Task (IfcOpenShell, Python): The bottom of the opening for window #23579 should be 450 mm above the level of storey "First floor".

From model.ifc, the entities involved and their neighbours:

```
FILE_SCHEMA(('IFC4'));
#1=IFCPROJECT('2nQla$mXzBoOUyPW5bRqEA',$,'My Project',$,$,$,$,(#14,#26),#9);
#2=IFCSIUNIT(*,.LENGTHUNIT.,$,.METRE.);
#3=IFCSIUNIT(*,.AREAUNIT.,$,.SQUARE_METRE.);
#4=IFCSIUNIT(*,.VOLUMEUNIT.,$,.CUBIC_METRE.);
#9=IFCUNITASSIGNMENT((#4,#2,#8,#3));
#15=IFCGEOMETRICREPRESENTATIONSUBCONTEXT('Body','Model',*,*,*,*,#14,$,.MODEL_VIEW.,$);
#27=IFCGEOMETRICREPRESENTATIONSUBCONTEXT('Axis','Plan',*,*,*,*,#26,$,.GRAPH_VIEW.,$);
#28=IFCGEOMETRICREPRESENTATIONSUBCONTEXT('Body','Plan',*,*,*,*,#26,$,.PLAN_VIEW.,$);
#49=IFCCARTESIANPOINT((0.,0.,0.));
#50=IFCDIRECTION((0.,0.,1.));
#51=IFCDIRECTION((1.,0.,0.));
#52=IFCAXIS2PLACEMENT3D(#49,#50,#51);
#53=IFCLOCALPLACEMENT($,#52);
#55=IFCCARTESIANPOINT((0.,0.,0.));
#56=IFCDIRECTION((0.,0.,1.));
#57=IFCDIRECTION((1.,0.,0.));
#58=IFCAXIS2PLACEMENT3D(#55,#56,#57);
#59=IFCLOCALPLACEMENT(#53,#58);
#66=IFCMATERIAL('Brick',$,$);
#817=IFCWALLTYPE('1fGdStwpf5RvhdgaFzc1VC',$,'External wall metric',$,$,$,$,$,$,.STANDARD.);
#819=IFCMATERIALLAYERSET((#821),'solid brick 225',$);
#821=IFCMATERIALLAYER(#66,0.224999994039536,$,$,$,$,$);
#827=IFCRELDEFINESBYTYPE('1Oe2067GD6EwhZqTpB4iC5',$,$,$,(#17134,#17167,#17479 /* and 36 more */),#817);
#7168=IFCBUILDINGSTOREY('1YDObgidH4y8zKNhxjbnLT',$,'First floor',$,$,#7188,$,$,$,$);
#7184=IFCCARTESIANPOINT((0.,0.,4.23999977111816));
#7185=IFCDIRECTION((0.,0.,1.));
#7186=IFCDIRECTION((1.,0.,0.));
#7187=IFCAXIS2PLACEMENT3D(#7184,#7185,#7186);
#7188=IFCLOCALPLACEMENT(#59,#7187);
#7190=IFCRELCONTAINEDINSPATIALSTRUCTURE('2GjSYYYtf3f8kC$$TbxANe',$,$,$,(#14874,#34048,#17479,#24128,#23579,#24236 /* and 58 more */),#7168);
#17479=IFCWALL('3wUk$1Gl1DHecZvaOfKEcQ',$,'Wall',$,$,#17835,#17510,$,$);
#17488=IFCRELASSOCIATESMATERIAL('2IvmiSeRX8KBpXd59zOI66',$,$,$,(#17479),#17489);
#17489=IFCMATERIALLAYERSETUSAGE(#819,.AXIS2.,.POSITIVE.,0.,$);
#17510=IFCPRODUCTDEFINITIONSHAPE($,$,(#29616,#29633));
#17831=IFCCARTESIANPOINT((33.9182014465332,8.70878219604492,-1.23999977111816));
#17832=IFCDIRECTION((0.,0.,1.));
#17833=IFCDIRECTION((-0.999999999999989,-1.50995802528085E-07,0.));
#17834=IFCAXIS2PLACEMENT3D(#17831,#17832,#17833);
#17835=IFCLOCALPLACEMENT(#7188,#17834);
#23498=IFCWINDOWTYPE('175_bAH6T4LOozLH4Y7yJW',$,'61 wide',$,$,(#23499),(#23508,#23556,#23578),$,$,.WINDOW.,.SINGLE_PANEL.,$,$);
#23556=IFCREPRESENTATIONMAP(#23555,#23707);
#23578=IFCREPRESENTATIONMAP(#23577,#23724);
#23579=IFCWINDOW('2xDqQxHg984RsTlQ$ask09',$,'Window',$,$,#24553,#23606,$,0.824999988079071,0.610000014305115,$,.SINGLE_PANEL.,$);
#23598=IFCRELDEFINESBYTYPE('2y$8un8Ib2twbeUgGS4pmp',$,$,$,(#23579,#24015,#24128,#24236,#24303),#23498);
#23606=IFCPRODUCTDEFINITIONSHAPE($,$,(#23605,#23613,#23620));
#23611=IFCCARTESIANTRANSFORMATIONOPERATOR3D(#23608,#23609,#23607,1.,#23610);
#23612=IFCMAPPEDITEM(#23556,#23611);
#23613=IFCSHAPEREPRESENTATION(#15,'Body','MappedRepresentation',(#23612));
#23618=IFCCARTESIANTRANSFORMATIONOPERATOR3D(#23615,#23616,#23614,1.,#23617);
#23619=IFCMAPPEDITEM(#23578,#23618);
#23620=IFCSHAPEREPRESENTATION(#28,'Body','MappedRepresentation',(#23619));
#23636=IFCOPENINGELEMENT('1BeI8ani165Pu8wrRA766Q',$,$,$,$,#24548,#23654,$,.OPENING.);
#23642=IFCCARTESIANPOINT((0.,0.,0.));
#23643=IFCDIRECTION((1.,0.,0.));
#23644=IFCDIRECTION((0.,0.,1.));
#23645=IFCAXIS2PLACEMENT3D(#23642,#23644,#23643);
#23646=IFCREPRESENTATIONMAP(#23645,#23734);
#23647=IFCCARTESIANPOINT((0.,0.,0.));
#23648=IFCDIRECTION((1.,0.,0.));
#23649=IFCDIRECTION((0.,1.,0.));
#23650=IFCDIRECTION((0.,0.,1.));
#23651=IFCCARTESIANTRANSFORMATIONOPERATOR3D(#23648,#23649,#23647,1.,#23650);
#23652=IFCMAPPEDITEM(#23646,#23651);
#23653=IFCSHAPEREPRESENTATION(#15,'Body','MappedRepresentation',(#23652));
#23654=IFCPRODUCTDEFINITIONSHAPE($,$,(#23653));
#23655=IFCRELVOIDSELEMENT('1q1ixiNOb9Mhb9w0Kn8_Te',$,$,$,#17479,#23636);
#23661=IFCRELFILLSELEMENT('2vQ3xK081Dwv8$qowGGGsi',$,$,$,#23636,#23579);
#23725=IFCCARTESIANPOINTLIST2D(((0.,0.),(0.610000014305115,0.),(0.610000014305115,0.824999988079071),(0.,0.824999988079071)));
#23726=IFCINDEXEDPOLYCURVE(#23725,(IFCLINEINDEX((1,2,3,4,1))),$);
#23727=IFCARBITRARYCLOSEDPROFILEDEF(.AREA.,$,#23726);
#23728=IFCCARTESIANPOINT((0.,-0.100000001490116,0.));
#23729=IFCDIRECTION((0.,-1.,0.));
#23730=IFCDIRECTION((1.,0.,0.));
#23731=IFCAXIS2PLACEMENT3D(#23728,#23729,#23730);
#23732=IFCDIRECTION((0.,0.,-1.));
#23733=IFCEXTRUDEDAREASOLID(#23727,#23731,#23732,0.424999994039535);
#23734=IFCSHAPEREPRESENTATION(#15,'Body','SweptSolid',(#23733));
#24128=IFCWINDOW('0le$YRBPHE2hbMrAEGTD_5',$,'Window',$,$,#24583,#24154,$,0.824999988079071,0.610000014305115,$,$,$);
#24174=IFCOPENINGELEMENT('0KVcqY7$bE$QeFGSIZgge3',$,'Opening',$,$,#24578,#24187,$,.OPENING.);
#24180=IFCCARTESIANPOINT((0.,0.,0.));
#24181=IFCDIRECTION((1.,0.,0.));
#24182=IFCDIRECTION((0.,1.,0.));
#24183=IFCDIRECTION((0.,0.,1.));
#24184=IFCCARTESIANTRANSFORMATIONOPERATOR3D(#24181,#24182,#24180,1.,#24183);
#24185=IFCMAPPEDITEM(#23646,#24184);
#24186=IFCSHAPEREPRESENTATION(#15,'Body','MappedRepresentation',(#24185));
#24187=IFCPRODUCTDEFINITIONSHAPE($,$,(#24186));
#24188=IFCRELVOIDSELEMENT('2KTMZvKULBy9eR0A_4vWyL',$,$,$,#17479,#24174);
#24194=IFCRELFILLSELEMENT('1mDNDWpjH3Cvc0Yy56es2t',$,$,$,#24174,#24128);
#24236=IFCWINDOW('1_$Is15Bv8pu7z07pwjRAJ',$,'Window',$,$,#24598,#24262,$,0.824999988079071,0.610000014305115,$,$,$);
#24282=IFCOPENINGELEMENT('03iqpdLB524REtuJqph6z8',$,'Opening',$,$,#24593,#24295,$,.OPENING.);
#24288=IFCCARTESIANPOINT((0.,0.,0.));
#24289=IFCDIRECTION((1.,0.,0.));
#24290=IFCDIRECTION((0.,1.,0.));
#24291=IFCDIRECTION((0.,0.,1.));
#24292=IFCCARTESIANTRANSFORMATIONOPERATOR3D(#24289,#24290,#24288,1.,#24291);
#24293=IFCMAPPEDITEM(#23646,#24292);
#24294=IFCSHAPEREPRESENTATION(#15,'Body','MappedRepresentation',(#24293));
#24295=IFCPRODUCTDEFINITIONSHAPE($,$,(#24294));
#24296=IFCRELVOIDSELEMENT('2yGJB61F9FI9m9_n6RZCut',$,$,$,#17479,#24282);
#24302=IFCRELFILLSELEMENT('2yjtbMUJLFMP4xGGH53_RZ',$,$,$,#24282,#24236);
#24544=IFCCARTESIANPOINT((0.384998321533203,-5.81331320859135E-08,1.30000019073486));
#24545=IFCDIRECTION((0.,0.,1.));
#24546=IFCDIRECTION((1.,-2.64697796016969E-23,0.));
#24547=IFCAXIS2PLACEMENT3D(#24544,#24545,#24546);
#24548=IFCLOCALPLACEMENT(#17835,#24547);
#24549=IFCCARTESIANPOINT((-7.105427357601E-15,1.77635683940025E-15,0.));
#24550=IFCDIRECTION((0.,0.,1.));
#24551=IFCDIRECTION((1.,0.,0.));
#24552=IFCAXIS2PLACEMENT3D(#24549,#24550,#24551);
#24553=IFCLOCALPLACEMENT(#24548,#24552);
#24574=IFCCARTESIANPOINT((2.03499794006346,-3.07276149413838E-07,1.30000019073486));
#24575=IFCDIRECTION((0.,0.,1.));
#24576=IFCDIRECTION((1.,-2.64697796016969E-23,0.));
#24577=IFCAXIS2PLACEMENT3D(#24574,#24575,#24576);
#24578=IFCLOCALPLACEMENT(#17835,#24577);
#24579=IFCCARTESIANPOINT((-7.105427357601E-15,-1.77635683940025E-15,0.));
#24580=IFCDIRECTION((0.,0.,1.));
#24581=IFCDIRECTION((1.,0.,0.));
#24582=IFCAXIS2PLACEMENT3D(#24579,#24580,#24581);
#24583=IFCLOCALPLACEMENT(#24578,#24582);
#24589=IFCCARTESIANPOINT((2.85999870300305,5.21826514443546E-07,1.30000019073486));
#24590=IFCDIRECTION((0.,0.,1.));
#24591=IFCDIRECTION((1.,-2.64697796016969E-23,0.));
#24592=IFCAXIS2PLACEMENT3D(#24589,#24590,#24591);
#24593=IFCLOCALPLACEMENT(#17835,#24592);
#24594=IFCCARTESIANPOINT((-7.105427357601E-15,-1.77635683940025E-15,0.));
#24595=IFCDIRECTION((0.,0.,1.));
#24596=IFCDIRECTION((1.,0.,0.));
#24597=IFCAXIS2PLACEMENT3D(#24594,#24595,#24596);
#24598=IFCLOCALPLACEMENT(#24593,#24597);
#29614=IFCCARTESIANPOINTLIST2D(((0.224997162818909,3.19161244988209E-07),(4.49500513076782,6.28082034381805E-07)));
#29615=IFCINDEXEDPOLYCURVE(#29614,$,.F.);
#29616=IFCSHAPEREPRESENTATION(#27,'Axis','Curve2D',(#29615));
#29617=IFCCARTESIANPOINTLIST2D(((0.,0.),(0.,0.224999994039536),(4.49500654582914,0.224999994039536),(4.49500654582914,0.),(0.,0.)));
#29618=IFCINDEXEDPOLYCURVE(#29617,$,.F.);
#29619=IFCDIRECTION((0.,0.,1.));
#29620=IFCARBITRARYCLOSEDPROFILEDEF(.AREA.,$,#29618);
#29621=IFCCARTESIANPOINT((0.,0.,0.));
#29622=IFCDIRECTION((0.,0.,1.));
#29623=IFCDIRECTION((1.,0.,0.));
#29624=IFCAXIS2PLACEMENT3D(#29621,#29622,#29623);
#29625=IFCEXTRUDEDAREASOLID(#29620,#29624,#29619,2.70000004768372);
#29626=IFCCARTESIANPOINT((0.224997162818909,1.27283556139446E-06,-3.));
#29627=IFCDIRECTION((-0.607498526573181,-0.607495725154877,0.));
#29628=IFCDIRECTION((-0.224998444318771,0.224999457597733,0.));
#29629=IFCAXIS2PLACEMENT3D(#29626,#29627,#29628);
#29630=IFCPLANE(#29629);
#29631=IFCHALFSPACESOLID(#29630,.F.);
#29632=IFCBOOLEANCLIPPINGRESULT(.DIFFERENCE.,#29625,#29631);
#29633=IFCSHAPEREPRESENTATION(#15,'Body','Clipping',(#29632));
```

```python
import numpy as np
import ifcopenshell
import ifcopenshell.api.geometry
import ifcopenshell.geom
import ifcopenshell.util.element
import ifcopenshell.util.placement
import ifcopenshell.util.shape
import ifcopenshell.util.unit

model = ifcopenshell.open("model.ifc")
unit_scale = ifcopenshell.util.unit.calculate_unit_scale(model)

window = model.by_guid("2xDqQxHg984RsTlQ$ask09")
opening = window.FillsVoids[0].RelatingOpeningElement
storey = ifcopenshell.util.element.get_container(window, ifc_class="IfcBuildingStorey")
level = ifcopenshell.util.placement.get_local_placement(storey.ObjectPlacement)[2, 3]

# The opening's origin need not be at the sill, so measure its lowest point.
shape = ifcopenshell.geom.create_shape(ifcopenshell.geom.settings(), opening)
bottom = ifcopenshell.util.shape.get_shape_bottom_elevation(shape, shape.geometry) / unit_scale
dz = level + 0.45 / unit_scale - bottom

shift = np.array([0.0, 0.0, dz])
# The window is placed relative to its opening, so it follows when the opening moves.
matrix = ifcopenshell.util.placement.get_local_placement(opening.ObjectPlacement)
matrix[:3, 3] += shift
ifcopenshell.api.geometry.edit_object_placement(
    model, product=opening, matrix=matrix, is_si=False, should_transform_children=True
)

print(f"moved by {dz * unit_scale:+.3f} m")

model.write("model_edited.ifc")
```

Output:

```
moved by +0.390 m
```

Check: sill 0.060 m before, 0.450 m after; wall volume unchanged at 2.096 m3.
